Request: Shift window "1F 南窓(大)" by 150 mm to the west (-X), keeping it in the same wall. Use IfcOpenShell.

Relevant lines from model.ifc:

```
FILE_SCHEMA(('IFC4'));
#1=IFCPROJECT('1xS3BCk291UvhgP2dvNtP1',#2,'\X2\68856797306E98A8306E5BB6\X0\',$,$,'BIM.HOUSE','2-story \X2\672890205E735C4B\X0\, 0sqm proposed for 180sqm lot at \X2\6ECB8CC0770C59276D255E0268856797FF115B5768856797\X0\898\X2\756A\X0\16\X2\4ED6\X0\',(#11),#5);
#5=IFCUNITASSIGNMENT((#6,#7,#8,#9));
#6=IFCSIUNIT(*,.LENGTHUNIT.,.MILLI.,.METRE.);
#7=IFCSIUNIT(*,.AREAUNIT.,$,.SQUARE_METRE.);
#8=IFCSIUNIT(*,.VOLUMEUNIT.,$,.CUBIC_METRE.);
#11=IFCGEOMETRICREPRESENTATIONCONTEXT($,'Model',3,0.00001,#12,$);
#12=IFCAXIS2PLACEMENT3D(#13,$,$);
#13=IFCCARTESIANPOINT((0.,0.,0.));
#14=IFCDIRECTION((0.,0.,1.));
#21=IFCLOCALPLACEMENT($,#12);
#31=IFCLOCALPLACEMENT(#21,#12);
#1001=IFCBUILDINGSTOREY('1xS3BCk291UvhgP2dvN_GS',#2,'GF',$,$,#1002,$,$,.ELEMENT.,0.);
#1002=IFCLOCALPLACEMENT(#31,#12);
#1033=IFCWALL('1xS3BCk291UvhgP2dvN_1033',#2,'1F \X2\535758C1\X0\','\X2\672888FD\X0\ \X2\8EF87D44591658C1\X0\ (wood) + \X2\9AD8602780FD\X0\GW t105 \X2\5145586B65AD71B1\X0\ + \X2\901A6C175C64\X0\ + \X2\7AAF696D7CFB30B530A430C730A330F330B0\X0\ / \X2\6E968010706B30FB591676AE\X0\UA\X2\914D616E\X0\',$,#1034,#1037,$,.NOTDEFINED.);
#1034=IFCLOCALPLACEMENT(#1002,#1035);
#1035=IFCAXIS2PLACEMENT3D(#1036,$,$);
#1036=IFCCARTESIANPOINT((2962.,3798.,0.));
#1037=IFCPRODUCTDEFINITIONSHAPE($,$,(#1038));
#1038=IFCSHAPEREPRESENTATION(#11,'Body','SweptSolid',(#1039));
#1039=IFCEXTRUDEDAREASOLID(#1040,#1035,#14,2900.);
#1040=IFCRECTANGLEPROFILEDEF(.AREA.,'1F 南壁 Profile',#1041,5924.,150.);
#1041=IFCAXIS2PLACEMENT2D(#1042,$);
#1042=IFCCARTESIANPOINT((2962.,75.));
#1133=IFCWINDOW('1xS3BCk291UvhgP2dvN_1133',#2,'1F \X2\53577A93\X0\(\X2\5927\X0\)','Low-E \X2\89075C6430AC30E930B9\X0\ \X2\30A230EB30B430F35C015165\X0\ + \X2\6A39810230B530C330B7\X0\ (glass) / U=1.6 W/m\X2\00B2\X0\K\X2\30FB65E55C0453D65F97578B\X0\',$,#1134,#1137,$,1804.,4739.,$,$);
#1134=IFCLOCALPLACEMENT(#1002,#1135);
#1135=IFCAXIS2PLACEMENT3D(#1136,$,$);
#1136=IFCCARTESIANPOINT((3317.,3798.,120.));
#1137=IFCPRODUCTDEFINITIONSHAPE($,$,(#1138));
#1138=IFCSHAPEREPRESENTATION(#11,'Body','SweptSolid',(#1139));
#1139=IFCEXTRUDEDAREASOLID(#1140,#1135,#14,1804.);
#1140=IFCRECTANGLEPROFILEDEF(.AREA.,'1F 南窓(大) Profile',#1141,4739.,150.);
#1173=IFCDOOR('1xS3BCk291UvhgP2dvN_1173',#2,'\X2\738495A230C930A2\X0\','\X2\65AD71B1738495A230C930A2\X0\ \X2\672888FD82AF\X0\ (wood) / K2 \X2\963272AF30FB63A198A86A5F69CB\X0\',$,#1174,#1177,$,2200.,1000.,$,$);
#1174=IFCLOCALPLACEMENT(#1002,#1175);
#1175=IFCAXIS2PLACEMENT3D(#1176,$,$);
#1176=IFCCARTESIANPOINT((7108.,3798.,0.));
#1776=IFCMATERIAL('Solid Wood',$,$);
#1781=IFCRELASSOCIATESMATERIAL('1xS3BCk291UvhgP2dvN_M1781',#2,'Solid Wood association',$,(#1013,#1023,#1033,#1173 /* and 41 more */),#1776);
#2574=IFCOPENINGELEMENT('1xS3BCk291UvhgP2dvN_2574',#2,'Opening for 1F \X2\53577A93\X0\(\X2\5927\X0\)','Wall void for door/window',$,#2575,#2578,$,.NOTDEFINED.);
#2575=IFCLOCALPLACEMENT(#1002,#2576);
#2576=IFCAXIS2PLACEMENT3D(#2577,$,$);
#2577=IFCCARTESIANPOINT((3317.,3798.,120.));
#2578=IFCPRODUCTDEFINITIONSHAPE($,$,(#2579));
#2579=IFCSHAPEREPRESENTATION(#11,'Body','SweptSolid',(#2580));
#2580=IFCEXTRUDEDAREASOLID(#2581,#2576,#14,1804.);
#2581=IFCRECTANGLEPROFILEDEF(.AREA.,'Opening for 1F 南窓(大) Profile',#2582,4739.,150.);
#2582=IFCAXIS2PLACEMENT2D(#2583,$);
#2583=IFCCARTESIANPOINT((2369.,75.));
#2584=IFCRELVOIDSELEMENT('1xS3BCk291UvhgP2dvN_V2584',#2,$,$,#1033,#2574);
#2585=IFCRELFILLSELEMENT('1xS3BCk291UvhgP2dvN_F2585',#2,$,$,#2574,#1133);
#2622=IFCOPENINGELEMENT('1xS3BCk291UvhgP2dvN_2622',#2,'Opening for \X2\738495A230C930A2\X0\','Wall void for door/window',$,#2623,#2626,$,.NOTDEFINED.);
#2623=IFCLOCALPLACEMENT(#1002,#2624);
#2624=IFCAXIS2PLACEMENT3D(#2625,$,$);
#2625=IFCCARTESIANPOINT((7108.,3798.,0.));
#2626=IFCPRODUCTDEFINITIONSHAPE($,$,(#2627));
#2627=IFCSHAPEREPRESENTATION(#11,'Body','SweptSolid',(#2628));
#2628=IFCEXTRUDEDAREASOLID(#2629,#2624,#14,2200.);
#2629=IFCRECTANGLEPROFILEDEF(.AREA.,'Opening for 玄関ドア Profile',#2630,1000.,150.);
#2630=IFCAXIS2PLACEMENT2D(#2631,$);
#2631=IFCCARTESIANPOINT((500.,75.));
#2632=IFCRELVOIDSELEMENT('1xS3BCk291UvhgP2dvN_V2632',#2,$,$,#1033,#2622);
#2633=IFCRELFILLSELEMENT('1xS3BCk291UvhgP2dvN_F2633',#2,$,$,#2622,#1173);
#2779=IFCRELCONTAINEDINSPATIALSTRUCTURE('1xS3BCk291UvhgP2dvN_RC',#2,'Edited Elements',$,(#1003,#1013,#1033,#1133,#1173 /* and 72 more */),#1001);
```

```python
import ifcopenshell
import ifcopenshell.api.geometry
import ifcopenshell.util.placement
import ifcopenshell.util.unit

model = ifcopenshell.open("model.ifc")
unit_scale = ifcopenshell.util.unit.calculate_unit_scale(model)

window = model.by_id(1133)
opening = window.FillsVoids[0].RelatingOpeningElement
wall = opening.VoidsElements[0].RelatingBuildingElement

wall_matrix = ifcopenshell.util.placement.get_local_placement(wall.ObjectPlacement)
shift = wall_matrix[:3, 0] * -0.15 / unit_scale
before = ifcopenshell.util.placement.get_local_placement(window.ObjectPlacement)[:3, 3].copy()

# The window is not placed relative to its opening, so move both.
for product in (opening, window):
    matrix = ifcopenshell.util.placement.get_local_placement(product.ObjectPlacement)
    matrix[:3, 3] += shift
    ifcopenshell.api.geometry.edit_object_placement(model, product=product, matrix=matrix, is_si=False)

after = ifcopenshell.util.placement.get_local_placement(window.ObjectPlacement)[:3, 3]
print("window moved by", (after - before).round(3) + 0.0)

model.write("model_rev.ifc")
```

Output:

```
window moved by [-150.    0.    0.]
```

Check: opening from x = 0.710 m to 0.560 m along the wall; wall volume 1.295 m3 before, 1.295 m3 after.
